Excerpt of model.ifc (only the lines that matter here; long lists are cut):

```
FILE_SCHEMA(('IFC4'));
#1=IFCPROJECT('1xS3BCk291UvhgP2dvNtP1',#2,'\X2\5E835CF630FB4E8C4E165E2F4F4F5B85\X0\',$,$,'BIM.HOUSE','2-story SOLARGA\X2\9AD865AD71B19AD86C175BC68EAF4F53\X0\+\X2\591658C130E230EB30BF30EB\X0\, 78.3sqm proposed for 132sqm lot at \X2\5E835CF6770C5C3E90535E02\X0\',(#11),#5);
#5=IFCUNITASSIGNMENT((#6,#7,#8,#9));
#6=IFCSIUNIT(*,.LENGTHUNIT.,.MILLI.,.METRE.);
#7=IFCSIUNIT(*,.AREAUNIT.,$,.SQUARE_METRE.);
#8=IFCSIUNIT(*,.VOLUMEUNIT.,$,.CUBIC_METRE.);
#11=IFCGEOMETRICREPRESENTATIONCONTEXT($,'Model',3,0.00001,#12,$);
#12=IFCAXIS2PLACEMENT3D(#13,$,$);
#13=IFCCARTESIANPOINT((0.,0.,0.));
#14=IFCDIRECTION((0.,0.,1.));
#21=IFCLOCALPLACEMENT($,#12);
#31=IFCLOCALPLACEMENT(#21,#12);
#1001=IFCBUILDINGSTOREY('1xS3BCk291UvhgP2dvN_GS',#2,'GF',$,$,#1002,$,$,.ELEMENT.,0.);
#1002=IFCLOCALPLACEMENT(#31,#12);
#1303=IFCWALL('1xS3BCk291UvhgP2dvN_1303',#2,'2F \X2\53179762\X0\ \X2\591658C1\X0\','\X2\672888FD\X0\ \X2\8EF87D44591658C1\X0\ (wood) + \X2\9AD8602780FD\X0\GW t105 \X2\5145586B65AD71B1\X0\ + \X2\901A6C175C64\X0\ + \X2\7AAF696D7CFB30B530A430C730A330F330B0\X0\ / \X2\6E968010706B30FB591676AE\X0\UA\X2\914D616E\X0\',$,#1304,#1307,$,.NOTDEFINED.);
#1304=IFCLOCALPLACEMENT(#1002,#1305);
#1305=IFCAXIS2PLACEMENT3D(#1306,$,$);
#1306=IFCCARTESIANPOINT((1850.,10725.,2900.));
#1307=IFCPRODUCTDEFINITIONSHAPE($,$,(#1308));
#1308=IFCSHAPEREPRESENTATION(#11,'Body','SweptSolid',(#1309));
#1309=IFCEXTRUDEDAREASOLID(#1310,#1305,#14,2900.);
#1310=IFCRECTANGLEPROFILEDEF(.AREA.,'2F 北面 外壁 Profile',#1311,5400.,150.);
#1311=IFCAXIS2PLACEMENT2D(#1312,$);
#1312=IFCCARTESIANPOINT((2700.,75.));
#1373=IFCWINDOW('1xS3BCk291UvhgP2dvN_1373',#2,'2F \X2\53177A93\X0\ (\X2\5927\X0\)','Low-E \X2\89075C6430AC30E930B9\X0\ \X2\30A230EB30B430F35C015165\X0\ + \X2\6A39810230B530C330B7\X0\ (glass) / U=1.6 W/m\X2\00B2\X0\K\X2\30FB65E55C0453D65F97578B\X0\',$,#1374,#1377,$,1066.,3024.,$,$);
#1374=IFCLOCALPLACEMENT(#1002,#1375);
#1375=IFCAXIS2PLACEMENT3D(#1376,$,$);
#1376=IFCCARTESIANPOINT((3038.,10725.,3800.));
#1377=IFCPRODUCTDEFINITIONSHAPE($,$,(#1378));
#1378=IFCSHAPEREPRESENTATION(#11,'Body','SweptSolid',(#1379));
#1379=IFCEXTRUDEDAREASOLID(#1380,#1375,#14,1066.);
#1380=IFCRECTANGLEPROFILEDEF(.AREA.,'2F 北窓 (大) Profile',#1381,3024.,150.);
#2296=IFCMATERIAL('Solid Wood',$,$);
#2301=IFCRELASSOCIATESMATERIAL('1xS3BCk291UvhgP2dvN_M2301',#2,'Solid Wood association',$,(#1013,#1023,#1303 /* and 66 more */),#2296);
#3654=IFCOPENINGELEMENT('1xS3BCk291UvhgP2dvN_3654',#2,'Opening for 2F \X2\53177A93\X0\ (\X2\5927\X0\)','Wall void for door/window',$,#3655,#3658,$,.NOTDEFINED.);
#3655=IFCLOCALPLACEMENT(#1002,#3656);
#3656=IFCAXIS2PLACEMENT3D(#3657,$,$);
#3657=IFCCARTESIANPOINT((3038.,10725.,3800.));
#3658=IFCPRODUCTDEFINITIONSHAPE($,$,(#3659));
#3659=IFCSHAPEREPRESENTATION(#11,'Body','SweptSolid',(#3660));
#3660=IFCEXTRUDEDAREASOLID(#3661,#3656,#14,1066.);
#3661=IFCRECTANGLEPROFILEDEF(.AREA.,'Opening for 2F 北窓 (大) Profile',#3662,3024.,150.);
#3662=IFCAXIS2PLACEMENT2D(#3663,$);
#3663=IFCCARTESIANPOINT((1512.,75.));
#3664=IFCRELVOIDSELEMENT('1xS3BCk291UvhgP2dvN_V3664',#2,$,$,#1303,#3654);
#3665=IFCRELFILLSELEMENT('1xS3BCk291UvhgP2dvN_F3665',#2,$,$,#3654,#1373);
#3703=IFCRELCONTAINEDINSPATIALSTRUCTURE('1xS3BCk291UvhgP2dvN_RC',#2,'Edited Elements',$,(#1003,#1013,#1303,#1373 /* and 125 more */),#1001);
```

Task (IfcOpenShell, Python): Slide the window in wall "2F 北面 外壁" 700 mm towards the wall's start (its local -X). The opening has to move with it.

```python
import ifcopenshell
import ifcopenshell.api.geometry
import ifcopenshell.util.placement
import ifcopenshell.util.unit

model = ifcopenshell.open("model.ifc")
unit_scale = ifcopenshell.util.unit.calculate_unit_scale(model)

window = model.by_guid("1xS3BCk291UvhgP2dvN_1373")
opening = window.FillsVoids[0].RelatingOpeningElement
wall = opening.VoidsElements[0].RelatingBuildingElement

wall_matrix = ifcopenshell.util.placement.get_local_placement(wall.ObjectPlacement)
shift = wall_matrix[:3, 0] * -0.7 / unit_scale
before = ifcopenshell.util.placement.get_local_placement(window.ObjectPlacement)[:3, 3].copy()

# The window is not placed relative to its opening, so move both.
for product in (opening, window):
    matrix = ifcopenshell.util.placement.get_local_placement(product.ObjectPlacement)
    matrix[:3, 3] += shift
    ifcopenshell.api.geometry.edit_object_placement(model, product=product, matrix=matrix, is_si=False)

after = ifcopenshell.util.placement.get_local_placement(window.ObjectPlacement)[:3, 3]
print("window moved by", (after - before).round(3) + 0.0)

model.write("model-out.ifc")
```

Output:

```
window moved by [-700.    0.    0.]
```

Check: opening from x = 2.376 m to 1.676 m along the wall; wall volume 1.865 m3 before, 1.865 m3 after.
